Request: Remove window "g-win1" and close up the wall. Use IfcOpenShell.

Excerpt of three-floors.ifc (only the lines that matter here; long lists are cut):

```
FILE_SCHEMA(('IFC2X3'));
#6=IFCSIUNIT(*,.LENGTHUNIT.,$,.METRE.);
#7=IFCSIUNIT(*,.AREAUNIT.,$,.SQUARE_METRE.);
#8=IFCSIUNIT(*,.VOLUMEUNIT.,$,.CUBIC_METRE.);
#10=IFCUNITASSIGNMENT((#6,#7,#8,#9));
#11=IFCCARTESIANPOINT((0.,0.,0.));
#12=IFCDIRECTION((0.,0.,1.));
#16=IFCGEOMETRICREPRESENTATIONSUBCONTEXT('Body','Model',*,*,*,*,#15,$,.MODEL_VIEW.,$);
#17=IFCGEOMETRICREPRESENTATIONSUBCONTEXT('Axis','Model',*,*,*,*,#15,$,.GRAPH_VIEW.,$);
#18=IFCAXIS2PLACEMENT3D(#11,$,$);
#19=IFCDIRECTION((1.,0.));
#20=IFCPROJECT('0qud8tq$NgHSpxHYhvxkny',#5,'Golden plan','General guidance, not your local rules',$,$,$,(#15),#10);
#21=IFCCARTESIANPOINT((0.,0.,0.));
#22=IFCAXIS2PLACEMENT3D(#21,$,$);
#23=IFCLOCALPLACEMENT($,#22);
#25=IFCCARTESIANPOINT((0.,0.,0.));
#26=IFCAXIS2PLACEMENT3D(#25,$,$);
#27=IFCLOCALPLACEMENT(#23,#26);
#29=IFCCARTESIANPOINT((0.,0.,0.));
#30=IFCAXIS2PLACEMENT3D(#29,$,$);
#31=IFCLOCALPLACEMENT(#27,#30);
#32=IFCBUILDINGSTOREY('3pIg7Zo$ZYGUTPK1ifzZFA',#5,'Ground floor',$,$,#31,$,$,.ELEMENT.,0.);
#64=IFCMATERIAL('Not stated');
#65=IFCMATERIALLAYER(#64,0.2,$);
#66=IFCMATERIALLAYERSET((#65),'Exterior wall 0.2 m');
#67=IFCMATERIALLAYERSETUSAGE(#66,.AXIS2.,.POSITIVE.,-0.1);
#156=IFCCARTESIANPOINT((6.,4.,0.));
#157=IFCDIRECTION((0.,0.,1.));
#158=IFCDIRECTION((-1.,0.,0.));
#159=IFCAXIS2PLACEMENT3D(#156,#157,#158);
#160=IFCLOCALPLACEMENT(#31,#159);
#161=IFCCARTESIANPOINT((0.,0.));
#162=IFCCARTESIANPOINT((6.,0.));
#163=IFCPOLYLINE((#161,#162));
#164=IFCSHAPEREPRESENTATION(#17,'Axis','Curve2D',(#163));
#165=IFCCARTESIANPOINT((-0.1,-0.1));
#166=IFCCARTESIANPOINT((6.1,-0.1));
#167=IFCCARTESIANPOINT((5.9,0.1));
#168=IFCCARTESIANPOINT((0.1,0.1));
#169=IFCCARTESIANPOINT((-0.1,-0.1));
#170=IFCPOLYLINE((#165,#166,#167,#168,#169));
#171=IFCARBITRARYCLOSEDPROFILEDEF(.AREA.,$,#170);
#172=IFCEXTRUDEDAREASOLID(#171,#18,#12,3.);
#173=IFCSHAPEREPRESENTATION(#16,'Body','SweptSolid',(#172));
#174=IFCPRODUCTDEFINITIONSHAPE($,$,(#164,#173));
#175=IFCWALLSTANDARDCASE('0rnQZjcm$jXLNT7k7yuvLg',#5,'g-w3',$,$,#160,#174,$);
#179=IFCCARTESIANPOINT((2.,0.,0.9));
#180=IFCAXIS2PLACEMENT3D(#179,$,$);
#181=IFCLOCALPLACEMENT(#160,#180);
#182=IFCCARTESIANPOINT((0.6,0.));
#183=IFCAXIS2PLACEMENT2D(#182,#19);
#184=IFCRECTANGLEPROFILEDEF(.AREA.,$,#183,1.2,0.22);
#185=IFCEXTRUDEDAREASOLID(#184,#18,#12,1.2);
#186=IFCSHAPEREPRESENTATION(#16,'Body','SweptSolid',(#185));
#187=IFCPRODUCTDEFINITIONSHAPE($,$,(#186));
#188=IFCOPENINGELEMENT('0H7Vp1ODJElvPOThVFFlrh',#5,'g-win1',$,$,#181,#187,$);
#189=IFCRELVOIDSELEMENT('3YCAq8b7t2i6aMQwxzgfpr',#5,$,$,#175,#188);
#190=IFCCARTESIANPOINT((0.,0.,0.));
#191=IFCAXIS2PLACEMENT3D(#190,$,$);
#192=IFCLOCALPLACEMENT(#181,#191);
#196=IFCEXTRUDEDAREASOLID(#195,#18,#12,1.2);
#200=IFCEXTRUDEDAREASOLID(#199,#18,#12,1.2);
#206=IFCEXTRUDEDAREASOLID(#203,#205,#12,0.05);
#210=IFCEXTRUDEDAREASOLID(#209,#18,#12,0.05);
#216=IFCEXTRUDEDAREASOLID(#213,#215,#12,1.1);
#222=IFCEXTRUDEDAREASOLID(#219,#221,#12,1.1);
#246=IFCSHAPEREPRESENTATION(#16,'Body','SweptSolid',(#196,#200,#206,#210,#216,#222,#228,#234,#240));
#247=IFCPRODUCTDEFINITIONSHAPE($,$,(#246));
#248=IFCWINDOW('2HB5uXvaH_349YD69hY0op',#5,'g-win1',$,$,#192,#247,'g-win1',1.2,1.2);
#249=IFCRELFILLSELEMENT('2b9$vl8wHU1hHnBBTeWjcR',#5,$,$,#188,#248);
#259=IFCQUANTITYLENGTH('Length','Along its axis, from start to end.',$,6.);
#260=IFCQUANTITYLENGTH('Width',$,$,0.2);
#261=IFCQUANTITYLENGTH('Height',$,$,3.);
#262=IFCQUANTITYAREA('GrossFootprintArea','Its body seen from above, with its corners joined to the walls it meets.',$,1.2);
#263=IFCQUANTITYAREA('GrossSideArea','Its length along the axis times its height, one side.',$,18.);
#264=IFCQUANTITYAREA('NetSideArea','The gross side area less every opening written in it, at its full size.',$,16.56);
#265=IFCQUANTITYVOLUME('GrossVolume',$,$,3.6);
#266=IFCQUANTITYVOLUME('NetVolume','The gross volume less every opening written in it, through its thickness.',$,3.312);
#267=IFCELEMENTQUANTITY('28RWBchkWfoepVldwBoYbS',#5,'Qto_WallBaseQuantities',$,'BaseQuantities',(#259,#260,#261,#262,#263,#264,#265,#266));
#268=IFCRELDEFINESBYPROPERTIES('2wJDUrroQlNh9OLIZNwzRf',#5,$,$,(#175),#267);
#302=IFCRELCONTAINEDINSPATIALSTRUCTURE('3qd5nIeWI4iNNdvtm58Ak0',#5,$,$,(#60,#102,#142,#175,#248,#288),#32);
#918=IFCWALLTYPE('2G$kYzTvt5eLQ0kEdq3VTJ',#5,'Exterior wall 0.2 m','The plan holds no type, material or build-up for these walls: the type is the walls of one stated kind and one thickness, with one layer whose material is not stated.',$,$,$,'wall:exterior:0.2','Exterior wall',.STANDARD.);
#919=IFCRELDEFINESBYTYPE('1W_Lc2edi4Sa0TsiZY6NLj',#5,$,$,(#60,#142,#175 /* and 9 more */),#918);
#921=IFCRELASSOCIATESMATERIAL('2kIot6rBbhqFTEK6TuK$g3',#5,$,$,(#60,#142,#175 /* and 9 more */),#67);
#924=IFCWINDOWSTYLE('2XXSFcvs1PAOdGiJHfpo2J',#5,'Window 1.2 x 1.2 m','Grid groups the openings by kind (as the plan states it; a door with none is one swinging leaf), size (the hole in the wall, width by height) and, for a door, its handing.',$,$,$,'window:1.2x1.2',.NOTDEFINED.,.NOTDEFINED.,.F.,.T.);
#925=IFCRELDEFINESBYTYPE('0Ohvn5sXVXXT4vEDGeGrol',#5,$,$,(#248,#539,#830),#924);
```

```python
import ifcopenshell
import ifcopenshell.api.feature
import ifcopenshell.api.pset
import ifcopenshell.api.root
import ifcopenshell.geom
import ifcopenshell.util.element
import ifcopenshell.util.shape
import ifcopenshell.util.unit

model = ifcopenshell.open("three-floors.ifc")
area_scale = ifcopenshell.util.unit.calculate_unit_scale(model, "AREAUNIT")
volume_scale = ifcopenshell.util.unit.calculate_unit_scale(model, "VOLUMEUNIT")
settings = ifcopenshell.geom.settings()


def volume(element):
    """Net volume in cubic metres, openings subtracted."""
    shape = ifcopenshell.geom.create_shape(settings, element)
    return ifcopenshell.util.shape.get_volume(shape.geometry)


window = model.by_guid("2HB5uXvaH_349YD69hY0op")
opening = window.FillsVoids[0].RelatingOpeningElement
wall = opening.VoidsElements[0].RelatingBuildingElement
before = volume(wall)

ifcopenshell.api.root.remove_product(model, product=window)
ifcopenshell.api.feature.remove_feature(model, feature=opening)

after = volume(wall)
thickness = 0.2  # wall thickness in metres

# Update the wall's stored quantities.
qto = model.by_id(ifcopenshell.util.element.get_pset(wall, "Qto_WallBaseQuantities", should_inherit=False)["id"])
ifcopenshell.api.pset.edit_qto(model, qto=qto, properties={
    "NetSideArea": after / thickness / area_scale,
    "NetVolume": after / volume_scale,
})

print(f"wall volume {before:.3f} -> {after:.3f} m3")

model.write("three-floors_rev.ifc")
```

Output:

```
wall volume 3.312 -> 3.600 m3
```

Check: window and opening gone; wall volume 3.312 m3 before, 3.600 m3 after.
